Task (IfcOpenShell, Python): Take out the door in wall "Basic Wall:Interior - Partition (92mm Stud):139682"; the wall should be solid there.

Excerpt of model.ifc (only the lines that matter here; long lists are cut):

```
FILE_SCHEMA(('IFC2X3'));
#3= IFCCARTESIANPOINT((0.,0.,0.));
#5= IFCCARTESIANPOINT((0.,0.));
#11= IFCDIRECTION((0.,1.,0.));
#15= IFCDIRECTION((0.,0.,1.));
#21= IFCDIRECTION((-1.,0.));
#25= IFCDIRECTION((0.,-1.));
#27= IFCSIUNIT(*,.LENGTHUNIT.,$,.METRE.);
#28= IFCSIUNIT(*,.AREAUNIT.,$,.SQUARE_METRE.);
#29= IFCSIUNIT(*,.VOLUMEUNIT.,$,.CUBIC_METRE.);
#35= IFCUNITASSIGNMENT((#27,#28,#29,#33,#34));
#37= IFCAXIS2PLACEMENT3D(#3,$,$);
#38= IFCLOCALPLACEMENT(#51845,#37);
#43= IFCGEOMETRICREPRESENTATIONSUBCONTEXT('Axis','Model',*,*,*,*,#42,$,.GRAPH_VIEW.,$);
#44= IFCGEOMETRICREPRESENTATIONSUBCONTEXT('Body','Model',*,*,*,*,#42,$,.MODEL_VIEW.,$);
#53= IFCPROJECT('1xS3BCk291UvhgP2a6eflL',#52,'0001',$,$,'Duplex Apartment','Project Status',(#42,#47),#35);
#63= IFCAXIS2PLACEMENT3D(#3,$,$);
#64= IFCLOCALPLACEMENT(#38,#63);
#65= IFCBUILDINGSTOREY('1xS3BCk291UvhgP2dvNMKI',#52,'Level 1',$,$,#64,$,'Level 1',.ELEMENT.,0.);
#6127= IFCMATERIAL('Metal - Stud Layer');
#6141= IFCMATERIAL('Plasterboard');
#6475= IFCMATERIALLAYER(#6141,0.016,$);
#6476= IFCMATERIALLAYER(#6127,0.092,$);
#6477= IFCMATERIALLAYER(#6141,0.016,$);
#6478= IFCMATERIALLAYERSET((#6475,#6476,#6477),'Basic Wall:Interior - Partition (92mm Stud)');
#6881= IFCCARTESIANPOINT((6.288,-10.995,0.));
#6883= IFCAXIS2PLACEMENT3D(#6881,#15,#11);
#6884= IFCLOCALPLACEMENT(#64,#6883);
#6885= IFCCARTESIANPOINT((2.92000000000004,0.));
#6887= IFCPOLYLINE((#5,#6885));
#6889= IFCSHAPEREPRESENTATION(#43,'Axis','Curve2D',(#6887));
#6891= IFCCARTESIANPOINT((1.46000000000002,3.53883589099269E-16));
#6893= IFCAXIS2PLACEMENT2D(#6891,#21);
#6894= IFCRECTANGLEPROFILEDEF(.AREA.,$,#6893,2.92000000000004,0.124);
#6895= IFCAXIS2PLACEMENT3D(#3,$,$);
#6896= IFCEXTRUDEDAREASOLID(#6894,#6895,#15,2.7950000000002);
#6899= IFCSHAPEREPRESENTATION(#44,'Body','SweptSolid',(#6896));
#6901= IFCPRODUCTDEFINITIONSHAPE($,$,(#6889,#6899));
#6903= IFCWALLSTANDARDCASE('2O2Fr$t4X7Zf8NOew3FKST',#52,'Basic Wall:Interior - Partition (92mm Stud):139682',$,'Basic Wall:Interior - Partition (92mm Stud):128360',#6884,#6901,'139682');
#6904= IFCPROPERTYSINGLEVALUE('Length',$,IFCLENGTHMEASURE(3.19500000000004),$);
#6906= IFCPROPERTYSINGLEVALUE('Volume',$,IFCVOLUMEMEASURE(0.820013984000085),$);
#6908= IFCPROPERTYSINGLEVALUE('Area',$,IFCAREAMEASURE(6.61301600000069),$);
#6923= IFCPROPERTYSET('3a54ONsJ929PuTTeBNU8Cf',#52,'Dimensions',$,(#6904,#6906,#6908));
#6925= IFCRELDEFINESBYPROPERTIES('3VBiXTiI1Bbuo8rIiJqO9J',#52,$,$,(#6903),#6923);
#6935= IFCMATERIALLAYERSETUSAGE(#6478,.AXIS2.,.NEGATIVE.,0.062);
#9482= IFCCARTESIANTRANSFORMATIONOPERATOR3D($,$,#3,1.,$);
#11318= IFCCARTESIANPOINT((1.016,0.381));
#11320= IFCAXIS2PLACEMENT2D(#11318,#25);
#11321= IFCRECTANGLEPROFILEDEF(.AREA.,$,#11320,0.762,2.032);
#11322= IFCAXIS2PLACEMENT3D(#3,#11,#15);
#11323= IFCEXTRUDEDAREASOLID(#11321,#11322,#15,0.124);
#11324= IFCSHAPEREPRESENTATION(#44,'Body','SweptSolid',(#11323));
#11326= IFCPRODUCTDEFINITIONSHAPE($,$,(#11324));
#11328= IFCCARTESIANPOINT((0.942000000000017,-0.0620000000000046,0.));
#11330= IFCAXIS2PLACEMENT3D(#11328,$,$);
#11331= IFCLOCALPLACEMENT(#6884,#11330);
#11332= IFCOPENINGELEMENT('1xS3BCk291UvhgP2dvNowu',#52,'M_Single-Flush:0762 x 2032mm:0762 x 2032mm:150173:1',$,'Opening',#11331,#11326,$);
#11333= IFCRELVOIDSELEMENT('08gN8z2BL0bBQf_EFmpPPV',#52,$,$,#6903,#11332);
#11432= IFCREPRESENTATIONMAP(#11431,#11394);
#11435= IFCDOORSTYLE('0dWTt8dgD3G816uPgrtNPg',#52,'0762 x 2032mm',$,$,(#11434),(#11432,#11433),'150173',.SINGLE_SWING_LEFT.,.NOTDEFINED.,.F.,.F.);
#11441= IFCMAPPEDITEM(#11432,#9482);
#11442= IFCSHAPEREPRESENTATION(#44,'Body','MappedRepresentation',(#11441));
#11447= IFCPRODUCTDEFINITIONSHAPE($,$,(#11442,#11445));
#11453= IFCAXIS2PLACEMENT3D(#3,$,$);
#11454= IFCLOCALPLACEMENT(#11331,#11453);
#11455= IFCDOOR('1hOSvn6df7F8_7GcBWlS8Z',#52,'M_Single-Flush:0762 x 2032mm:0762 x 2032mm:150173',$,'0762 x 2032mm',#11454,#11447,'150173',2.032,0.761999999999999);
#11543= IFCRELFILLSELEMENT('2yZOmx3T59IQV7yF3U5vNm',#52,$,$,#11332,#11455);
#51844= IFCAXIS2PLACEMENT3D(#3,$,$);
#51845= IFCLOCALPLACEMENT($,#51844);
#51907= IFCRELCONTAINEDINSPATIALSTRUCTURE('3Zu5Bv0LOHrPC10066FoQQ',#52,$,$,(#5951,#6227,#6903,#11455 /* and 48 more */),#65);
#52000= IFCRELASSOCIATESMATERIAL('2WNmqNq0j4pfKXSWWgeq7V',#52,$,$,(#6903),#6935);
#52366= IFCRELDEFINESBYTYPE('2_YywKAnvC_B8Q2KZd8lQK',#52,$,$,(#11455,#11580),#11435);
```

```python
import ifcopenshell
import ifcopenshell.api.feature
import ifcopenshell.api.pset
import ifcopenshell.api.root
import ifcopenshell.geom
import ifcopenshell.util.element
import ifcopenshell.util.shape
import ifcopenshell.util.unit

model = ifcopenshell.open("model.ifc")
area_scale = ifcopenshell.util.unit.calculate_unit_scale(model, "AREAUNIT")
volume_scale = ifcopenshell.util.unit.calculate_unit_scale(model, "VOLUMEUNIT")
settings = ifcopenshell.geom.settings()


def volume(element):
    """Net volume in cubic metres, openings subtracted."""
    shape = ifcopenshell.geom.create_shape(settings, element)
    return ifcopenshell.util.shape.get_volume(shape.geometry)


door = model.by_guid("1hOSvn6df7F8_7GcBWlS8Z")
opening = door.FillsVoids[0].RelatingOpeningElement
wall = opening.VoidsElements[0].RelatingBuildingElement
before = volume(wall)

ifcopenshell.api.root.remove_product(model, product=door)
ifcopenshell.api.feature.remove_feature(model, feature=opening)

after = volume(wall)
thickness = 0.124  # wall thickness in metres

# Update the wall's stored quantities.
pset = model.by_id(ifcopenshell.util.element.get_pset(wall, "Dimensions", should_inherit=False)["id"])
ifcopenshell.api.pset.edit_pset(model, pset=pset, properties={
    "Volume": model.create_entity("IfcVolumeMeasure", after / volume_scale),
    "Area": model.create_entity("IfcAreaMeasure", after / thickness / area_scale),
})

print(f"wall volume {before:.3f} -> {after:.3f} m3")

model.write("model_rev.ifc")
```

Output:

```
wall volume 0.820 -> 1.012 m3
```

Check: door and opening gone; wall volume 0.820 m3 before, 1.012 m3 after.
